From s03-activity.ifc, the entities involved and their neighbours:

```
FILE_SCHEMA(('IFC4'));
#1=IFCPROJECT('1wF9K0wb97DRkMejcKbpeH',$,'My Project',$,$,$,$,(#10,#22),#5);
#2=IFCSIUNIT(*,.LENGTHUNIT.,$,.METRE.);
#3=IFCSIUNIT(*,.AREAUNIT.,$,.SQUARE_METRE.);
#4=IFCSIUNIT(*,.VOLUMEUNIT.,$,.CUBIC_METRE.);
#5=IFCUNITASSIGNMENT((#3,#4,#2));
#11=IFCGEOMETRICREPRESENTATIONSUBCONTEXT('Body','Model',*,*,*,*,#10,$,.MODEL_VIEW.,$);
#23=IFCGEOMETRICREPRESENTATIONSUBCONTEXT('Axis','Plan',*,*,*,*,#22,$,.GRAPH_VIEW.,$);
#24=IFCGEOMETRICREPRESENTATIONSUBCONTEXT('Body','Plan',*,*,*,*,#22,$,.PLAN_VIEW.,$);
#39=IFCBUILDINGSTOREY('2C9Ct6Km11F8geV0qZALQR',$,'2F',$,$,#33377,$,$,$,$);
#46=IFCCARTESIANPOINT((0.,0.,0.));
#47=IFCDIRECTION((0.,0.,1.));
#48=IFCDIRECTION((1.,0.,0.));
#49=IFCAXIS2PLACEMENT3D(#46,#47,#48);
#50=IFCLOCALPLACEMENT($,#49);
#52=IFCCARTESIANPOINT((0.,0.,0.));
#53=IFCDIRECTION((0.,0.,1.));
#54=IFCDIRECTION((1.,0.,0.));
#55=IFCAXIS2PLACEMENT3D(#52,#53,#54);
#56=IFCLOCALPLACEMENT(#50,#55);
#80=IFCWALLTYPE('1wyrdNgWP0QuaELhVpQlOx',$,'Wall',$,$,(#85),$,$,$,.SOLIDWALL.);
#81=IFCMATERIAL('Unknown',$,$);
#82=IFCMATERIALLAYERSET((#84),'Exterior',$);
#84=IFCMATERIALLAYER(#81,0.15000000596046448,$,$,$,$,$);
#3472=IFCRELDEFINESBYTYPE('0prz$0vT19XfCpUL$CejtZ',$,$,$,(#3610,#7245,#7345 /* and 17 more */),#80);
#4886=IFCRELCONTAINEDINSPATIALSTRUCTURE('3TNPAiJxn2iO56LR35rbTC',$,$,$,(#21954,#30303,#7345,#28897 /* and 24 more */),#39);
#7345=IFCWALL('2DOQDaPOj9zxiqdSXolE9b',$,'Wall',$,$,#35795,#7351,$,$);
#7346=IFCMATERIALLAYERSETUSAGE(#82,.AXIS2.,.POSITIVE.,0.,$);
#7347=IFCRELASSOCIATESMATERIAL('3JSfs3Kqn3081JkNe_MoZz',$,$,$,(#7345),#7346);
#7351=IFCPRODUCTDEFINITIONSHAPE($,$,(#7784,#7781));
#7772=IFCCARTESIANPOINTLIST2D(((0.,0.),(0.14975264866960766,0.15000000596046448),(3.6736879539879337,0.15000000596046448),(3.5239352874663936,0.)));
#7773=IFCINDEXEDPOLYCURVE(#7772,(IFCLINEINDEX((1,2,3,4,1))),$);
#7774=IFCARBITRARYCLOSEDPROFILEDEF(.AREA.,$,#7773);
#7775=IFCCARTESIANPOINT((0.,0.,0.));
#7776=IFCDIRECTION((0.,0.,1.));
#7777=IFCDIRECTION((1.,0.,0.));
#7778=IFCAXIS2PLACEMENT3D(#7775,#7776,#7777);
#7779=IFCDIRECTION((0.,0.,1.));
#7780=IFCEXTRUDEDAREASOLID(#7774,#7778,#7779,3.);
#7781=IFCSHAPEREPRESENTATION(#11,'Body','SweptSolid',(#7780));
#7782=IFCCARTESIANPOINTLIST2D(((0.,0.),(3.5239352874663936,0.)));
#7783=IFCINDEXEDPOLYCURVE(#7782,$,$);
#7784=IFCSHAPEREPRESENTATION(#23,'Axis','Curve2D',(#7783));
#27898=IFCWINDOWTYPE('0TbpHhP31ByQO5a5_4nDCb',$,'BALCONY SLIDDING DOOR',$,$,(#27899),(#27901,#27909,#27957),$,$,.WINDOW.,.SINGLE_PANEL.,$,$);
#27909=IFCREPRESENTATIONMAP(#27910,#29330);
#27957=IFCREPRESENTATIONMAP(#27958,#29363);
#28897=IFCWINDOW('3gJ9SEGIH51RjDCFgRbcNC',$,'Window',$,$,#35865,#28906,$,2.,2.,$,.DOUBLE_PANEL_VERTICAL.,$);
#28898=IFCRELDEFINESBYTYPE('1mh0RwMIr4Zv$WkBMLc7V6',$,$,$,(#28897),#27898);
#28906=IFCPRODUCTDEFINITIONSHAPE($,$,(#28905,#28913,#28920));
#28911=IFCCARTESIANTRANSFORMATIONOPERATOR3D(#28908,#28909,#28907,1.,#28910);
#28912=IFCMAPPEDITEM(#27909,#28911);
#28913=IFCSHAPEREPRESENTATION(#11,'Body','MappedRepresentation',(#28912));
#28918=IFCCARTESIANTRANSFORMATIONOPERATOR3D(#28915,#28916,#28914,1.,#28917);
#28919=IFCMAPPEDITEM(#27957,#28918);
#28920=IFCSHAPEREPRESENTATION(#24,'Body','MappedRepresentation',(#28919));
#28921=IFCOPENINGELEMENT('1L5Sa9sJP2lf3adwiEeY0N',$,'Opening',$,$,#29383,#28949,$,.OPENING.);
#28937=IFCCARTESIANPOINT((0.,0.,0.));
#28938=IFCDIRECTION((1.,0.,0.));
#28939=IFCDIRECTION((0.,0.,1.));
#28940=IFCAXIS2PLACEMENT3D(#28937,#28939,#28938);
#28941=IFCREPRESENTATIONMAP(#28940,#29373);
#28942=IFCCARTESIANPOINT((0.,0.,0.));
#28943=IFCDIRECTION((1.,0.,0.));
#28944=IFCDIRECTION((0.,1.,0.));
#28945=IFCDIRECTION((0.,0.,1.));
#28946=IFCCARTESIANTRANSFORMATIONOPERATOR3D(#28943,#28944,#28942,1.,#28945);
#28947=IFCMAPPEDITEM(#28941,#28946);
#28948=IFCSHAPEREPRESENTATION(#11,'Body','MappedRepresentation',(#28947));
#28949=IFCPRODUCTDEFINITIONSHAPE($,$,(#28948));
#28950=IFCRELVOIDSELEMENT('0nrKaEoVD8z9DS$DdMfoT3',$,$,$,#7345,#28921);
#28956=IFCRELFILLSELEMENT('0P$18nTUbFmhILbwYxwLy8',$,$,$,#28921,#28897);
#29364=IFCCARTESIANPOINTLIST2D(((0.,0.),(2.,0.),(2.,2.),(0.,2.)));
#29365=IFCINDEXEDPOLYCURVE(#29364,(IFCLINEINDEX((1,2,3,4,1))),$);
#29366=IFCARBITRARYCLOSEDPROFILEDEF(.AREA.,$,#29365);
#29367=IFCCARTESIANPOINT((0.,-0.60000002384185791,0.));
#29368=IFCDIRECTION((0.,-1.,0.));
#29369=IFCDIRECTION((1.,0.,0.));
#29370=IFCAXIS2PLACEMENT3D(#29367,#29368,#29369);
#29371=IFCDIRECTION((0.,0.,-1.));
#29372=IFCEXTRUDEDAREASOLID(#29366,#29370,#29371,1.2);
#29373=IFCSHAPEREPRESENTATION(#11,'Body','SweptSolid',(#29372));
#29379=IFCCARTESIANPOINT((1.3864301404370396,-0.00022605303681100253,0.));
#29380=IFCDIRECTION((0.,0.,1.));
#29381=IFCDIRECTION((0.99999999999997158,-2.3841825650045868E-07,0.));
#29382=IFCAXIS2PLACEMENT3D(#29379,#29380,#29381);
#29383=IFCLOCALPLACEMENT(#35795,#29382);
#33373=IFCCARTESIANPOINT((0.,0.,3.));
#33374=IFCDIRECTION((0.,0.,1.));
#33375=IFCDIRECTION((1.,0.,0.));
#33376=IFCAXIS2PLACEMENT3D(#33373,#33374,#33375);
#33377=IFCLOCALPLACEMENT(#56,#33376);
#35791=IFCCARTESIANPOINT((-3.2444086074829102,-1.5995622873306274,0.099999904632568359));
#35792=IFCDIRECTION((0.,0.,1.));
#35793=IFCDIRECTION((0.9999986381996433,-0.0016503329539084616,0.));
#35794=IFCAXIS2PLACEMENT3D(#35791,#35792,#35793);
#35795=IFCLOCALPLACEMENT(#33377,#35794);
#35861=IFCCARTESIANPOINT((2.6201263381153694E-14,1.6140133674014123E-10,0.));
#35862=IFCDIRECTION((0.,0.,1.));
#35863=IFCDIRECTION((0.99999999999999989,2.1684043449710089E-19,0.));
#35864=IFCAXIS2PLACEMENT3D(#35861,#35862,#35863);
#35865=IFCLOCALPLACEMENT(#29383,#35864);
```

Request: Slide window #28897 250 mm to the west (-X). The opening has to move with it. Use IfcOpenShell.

```python
import ifcopenshell
import ifcopenshell.api.geometry
import ifcopenshell.util.placement
import ifcopenshell.util.unit

model = ifcopenshell.open("s03-activity.ifc")
unit_scale = ifcopenshell.util.unit.calculate_unit_scale(model)

window = model.by_guid("3gJ9SEGIH51RjDCFgRbcNC")
opening = window.FillsVoids[0].RelatingOpeningElement
wall = opening.VoidsElements[0].RelatingBuildingElement

wall_matrix = ifcopenshell.util.placement.get_local_placement(wall.ObjectPlacement)
shift = wall_matrix[:3, 0] * -0.25 / unit_scale
before = ifcopenshell.util.placement.get_local_placement(window.ObjectPlacement)[:3, 3].copy()

# The window is placed relative to its opening, so it follows when the opening moves.
matrix = ifcopenshell.util.placement.get_local_placement(opening.ObjectPlacement)
matrix[:3, 3] += shift
ifcopenshell.api.geometry.edit_object_placement(
    model, product=opening, matrix=matrix, is_si=False, should_transform_children=True
)

after = ifcopenshell.util.placement.get_local_placement(window.ObjectPlacement)[:3, 3]
print("window moved by", (after - before).round(3) + 0.0)

model.write("s03-activity_updated.ifc")
```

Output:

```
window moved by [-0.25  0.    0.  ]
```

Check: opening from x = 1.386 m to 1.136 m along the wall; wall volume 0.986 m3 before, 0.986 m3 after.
